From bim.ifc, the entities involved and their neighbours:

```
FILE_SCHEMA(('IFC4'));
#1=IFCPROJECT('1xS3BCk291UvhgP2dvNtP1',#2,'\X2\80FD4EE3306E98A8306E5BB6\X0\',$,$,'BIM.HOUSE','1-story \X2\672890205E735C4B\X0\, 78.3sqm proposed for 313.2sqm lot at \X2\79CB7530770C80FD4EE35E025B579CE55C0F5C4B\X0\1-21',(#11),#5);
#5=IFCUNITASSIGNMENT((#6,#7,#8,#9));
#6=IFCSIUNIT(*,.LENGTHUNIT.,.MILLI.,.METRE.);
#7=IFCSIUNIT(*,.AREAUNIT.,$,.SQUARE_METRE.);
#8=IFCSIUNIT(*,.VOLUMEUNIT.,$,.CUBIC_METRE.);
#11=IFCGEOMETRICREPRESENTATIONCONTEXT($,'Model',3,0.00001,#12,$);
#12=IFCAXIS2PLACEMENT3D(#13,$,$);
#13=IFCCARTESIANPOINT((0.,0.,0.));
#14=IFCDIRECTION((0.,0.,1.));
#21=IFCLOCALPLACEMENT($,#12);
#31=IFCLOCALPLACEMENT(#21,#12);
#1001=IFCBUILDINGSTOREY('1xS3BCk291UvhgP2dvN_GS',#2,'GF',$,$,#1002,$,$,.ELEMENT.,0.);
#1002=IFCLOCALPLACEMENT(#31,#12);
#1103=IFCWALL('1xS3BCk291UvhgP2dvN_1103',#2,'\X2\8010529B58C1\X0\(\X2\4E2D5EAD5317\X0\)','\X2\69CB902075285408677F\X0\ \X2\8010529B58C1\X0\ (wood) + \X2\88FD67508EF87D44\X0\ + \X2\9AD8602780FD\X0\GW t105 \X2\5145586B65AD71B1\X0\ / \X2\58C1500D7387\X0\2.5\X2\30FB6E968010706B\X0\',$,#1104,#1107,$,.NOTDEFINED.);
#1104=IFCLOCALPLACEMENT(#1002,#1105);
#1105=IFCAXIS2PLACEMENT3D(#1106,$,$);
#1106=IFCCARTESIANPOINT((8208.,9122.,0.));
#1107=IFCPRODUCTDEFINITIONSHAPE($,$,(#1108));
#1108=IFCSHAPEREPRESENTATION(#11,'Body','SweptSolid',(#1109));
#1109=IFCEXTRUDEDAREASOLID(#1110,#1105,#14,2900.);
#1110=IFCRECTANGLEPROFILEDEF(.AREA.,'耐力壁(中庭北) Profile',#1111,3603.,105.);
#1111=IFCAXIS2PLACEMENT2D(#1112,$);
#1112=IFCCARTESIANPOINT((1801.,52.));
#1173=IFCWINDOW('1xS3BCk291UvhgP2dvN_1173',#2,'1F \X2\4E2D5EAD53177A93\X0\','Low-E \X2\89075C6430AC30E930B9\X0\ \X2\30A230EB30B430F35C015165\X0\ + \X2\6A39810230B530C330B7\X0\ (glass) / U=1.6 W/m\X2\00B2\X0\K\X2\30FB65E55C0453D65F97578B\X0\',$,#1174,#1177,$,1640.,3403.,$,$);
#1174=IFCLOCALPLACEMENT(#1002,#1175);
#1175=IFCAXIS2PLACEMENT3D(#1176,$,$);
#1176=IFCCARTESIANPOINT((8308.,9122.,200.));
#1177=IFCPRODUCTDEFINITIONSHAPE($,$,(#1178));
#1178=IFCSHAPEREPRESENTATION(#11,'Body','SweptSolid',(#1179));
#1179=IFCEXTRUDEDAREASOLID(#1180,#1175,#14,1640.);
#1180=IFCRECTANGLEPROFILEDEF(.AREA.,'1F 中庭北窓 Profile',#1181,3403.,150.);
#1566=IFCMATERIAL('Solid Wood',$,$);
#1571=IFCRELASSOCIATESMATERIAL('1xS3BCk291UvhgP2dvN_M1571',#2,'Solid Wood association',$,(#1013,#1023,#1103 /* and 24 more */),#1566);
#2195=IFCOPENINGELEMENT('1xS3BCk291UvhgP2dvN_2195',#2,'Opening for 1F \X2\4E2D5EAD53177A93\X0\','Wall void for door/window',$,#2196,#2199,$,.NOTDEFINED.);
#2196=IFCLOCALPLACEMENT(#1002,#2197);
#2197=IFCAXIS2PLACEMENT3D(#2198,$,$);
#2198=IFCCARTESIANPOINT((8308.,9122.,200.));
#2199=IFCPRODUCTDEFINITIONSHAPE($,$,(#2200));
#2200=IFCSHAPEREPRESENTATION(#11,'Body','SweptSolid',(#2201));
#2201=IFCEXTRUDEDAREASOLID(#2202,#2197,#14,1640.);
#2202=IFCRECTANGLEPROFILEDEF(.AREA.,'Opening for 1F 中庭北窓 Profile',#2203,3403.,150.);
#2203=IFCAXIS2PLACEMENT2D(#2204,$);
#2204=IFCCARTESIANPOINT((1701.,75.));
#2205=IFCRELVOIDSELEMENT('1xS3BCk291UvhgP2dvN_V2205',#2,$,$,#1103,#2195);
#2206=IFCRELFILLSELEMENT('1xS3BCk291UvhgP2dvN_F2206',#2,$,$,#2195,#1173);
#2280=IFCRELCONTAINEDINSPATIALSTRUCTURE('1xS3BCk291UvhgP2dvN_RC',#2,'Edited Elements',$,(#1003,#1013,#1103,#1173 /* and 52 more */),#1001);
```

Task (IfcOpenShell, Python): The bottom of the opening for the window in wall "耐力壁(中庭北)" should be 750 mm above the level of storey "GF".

```python
import numpy as np
import ifcopenshell
import ifcopenshell.api.geometry
import ifcopenshell.geom
import ifcopenshell.util.element
import ifcopenshell.util.placement
import ifcopenshell.util.shape
import ifcopenshell.util.unit

model = ifcopenshell.open("bim.ifc")
unit_scale = ifcopenshell.util.unit.calculate_unit_scale(model)

window = model.by_guid("1xS3BCk291UvhgP2dvN_1173")
opening = window.FillsVoids[0].RelatingOpeningElement
storey = ifcopenshell.util.element.get_container(window, ifc_class="IfcBuildingStorey")
level = ifcopenshell.util.placement.get_local_placement(storey.ObjectPlacement)[2, 3]

# The opening's origin need not be at the sill, so measure its lowest point.
shape = ifcopenshell.geom.create_shape(ifcopenshell.geom.settings(), opening)
bottom = ifcopenshell.util.shape.get_shape_bottom_elevation(shape, shape.geometry) / unit_scale
dz = level + 0.75 / unit_scale - bottom

shift = np.array([0.0, 0.0, dz])
# The window is not placed relative to its opening, so move both.
for product in (opening, window):
    matrix = ifcopenshell.util.placement.get_local_placement(product.ObjectPlacement)
    matrix[:3, 3] += shift
    ifcopenshell.api.geometry.edit_object_placement(model, product=product, matrix=matrix, is_si=False)

print(f"moved by {dz * unit_scale:+.3f} m")

model.write("bim_edited.ifc")
```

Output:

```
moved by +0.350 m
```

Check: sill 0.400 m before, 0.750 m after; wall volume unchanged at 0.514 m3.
